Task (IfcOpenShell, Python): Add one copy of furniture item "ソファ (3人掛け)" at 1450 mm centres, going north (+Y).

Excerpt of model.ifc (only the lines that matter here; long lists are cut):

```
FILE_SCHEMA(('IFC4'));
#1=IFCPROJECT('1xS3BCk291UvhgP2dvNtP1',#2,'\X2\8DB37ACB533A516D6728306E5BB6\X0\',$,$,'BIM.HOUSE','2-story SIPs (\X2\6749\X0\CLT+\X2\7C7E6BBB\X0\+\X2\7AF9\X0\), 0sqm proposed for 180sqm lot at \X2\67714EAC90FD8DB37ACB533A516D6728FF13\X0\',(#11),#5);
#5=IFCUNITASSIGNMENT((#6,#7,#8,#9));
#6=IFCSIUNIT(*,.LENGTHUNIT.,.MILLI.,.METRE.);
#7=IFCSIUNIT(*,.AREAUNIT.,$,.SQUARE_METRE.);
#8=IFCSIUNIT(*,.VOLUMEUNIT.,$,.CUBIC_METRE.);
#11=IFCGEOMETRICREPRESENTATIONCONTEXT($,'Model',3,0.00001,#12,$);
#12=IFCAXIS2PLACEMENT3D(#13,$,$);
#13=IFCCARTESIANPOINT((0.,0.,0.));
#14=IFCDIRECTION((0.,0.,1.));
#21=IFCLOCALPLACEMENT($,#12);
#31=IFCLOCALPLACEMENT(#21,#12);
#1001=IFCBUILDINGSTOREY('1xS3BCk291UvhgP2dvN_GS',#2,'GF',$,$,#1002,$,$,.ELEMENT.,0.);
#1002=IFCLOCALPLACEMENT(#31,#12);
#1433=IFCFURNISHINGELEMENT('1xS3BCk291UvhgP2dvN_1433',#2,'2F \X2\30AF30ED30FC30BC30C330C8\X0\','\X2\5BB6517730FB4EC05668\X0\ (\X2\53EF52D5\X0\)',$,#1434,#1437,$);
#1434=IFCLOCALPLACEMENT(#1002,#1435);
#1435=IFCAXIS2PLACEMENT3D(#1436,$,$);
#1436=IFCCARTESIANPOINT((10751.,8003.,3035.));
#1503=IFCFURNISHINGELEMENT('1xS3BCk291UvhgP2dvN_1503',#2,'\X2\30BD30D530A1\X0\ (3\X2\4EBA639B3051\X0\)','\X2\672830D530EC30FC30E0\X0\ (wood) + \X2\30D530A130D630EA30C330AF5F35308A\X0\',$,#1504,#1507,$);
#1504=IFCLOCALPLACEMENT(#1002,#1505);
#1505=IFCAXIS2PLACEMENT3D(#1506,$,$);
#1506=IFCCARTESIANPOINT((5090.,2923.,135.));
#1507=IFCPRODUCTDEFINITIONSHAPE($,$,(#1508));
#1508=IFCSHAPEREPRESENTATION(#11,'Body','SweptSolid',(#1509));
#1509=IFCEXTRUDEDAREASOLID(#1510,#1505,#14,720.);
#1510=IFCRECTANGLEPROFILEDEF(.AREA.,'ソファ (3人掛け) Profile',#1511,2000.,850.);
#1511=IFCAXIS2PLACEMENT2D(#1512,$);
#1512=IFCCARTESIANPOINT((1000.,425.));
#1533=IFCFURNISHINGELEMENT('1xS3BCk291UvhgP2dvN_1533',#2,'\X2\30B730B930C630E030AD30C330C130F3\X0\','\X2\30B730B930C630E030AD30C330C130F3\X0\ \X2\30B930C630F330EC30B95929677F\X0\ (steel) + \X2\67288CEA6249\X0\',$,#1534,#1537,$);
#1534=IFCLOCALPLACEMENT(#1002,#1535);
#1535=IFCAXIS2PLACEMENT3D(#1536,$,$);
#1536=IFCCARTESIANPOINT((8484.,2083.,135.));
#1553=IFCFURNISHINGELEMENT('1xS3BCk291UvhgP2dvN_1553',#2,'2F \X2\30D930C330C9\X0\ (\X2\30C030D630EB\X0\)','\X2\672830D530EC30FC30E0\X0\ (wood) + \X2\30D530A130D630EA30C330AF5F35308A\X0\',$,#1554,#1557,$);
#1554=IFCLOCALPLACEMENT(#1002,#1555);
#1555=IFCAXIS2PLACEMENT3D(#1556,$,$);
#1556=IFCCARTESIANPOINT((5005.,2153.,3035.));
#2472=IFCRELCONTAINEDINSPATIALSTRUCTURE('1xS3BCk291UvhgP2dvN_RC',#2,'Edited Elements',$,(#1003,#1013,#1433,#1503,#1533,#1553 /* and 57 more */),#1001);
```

```python
import numpy as np
import ifcopenshell
import ifcopenshell.api.geometry
import ifcopenshell.api.root
import ifcopenshell.util.element
import ifcopenshell.util.placement
import ifcopenshell.util.unit

model = ifcopenshell.open("model.ifc")
unit_scale = ifcopenshell.util.unit.calculate_unit_scale(model)


def reuse_history(source, copy):
    """copy_class also copies each property set's owner history, people and application; keep the originals."""
    for rel in copy.IsDefinedBy:
        if rel.is_a("IfcRelDefinesByProperties") and (history := rel.RelatingPropertyDefinition.OwnerHistory):
            rel.RelatingPropertyDefinition.OwnerHistory = source.OwnerHistory
            ifcopenshell.util.element.remove_deep2(model, history)


source = model.by_guid("1xS3BCk291UvhgP2dvN_1503")
base = ifcopenshell.util.placement.get_local_placement(source.ObjectPlacement)
step = np.array([0.0, 1.0, 0.0]) * 1.45 / unit_scale

for i in range(1, 2):
    copy = ifcopenshell.api.root.copy_class(model, product=source)
    copy.Representation = ifcopenshell.util.element.copy_deep(
        model, source.Representation, exclude=["IfcGeometricRepresentationContext", "IfcRepresentationMap"]
    )
    reuse_history(source, copy)
    matrix = base.copy()
    matrix[:3, 3] += i * step
    print("added at", matrix[:3, 3].round(3) + 0.0)
    ifcopenshell.api.geometry.edit_object_placement(model, product=copy, matrix=matrix, is_si=False)

model.write("model_updated.ifc")
```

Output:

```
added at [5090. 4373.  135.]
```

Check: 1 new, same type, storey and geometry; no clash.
